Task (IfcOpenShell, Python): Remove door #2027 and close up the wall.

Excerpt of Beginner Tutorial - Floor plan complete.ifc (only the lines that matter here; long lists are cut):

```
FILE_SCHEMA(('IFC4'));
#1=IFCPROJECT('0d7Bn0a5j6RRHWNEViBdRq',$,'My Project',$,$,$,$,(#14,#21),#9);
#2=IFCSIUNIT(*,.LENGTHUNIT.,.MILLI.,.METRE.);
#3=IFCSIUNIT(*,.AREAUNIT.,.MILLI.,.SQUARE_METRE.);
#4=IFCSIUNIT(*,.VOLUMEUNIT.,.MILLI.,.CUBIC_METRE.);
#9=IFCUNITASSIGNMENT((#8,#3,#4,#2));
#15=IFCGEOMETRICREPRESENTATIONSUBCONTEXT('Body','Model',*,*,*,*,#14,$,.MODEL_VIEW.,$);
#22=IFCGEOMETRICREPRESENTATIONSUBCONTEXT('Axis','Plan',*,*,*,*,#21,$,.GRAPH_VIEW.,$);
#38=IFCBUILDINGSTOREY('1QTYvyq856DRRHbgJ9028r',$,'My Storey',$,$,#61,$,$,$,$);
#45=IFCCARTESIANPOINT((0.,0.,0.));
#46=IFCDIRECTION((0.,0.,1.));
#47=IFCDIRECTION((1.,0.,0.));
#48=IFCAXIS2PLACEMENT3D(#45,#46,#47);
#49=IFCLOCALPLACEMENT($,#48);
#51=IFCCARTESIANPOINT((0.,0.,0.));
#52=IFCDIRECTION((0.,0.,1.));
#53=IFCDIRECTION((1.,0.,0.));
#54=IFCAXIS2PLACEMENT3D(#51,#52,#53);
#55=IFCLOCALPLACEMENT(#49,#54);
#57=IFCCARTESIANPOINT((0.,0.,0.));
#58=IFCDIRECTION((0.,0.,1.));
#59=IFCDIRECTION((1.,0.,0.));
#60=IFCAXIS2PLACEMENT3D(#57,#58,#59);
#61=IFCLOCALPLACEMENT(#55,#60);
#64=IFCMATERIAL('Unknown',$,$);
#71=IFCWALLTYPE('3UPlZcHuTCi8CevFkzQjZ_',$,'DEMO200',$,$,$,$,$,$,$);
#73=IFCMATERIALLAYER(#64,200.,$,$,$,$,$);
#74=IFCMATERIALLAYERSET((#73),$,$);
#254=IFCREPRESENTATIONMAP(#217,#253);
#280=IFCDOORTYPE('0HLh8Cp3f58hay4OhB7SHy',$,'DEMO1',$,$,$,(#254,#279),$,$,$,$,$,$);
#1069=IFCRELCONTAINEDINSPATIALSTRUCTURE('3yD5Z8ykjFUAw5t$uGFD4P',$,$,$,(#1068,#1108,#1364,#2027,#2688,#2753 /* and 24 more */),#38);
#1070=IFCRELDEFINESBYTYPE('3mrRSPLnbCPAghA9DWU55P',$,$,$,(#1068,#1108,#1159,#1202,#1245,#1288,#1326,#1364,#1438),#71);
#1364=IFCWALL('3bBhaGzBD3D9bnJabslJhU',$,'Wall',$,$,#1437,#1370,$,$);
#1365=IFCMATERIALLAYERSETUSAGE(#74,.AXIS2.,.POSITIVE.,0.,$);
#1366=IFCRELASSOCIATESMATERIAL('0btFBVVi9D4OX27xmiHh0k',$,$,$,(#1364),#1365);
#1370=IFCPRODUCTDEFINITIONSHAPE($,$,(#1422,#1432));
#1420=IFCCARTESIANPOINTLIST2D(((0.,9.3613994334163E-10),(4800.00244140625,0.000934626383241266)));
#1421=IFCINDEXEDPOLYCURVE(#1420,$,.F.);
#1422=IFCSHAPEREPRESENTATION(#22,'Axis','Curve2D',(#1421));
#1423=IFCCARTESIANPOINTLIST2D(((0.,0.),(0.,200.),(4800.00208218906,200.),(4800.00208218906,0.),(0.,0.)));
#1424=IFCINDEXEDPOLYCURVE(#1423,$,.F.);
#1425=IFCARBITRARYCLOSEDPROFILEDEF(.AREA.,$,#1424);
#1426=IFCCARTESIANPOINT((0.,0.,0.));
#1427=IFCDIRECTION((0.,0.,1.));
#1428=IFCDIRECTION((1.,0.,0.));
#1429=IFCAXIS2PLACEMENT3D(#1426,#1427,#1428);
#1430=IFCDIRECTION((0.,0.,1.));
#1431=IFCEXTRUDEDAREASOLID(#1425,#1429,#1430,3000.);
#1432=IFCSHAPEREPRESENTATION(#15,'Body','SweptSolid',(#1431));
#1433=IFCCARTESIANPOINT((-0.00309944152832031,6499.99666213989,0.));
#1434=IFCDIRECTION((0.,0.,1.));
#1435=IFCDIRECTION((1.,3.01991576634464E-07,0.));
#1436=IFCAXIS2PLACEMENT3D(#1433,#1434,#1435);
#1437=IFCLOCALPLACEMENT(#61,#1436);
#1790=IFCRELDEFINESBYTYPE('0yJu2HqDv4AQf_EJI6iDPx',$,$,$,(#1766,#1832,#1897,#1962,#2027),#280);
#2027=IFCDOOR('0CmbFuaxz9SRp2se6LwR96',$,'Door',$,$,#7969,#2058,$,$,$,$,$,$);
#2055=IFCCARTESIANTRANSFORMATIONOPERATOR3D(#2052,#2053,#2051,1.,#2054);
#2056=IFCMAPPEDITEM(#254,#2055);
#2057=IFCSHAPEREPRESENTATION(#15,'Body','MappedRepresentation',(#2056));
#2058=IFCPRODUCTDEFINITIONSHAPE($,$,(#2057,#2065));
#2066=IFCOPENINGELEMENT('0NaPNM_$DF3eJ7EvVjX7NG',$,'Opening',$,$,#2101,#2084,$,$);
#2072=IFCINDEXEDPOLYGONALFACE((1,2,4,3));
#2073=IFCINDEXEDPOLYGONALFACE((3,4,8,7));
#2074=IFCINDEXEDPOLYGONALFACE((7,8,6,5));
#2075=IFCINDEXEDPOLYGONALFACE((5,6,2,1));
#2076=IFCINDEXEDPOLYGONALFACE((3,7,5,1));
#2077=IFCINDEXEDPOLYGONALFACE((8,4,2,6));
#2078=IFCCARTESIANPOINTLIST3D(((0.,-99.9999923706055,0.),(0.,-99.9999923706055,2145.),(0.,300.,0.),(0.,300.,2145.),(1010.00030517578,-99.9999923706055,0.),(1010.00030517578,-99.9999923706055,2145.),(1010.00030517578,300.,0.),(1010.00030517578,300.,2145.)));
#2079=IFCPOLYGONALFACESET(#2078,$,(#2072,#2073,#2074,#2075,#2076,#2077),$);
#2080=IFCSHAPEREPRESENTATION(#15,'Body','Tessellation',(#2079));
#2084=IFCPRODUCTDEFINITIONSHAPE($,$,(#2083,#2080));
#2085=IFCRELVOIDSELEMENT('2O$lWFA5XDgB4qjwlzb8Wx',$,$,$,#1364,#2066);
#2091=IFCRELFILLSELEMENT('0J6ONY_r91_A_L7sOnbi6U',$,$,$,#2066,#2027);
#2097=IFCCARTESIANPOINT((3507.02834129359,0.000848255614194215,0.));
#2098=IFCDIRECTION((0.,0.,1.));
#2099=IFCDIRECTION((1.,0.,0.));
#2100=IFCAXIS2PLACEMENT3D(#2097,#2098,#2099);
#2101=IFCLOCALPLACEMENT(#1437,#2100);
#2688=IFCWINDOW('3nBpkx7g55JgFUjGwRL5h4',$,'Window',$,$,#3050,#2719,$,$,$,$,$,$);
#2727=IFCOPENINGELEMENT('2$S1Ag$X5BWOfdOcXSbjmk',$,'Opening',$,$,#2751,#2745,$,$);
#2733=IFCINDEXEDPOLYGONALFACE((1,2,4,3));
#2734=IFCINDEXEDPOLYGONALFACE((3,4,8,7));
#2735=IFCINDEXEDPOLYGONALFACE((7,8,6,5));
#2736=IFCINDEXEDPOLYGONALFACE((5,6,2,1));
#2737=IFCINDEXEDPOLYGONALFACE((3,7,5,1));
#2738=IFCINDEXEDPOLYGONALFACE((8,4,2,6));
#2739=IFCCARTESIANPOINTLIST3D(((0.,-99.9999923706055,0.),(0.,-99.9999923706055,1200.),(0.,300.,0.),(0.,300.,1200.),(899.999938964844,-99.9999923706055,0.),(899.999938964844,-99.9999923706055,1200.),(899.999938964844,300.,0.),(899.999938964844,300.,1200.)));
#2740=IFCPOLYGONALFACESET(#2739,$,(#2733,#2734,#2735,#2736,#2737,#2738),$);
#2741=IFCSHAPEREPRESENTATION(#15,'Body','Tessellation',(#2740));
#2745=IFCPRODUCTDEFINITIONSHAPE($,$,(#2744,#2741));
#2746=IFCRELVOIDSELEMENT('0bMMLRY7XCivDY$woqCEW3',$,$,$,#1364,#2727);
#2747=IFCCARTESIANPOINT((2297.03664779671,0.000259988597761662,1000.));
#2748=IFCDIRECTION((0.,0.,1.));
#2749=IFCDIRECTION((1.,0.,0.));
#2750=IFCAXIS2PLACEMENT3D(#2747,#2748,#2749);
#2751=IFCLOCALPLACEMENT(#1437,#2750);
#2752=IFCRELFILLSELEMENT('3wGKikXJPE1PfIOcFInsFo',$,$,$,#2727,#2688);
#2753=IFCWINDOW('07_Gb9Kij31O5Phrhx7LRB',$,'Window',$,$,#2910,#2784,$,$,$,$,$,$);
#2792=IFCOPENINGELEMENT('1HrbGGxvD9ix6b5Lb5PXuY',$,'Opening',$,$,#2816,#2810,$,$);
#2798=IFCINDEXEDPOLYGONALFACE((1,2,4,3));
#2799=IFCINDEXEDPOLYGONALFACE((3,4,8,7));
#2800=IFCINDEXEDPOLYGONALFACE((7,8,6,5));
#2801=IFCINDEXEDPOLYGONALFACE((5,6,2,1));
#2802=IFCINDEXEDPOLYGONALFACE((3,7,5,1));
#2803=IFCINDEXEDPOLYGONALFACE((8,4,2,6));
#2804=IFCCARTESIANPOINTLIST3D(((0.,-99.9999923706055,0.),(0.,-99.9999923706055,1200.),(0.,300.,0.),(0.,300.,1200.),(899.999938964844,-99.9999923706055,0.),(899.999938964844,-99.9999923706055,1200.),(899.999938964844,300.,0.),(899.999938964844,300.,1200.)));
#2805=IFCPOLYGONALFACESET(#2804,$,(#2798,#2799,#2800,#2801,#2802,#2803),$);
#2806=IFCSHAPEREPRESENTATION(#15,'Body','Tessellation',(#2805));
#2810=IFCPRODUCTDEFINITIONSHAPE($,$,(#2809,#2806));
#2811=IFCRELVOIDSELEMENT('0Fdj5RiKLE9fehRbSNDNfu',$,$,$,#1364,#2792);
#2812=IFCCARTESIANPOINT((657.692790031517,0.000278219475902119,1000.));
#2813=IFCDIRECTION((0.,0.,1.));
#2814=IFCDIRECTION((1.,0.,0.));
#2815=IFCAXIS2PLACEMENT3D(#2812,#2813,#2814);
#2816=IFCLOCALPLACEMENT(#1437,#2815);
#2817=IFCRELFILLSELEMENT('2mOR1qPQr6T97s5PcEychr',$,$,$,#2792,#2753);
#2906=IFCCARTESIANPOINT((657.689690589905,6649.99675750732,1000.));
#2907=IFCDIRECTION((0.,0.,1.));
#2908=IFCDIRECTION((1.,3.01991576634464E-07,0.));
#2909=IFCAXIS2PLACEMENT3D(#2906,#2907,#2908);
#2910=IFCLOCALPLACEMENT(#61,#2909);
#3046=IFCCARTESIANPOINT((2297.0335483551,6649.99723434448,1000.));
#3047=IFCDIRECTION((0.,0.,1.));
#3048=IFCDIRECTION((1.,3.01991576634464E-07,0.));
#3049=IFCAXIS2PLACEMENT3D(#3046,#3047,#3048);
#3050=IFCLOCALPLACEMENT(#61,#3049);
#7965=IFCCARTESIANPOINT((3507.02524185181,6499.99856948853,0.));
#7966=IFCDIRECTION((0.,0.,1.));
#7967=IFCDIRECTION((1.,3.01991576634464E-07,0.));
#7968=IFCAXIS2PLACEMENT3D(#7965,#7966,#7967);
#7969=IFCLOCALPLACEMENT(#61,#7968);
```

```python
import ifcopenshell
import ifcopenshell.api.feature
import ifcopenshell.api.root
import ifcopenshell.geom
import ifcopenshell.util.shape

model = ifcopenshell.open("Beginner Tutorial - Floor plan complete.ifc")
settings = ifcopenshell.geom.settings()


def volume(element):
    """Net volume in cubic metres, openings subtracted."""
    shape = ifcopenshell.geom.create_shape(settings, element)
    return ifcopenshell.util.shape.get_volume(shape.geometry)


door = model.by_guid("0CmbFuaxz9SRp2se6LwR96")
opening = door.FillsVoids[0].RelatingOpeningElement
wall = opening.VoidsElements[0].RelatingBuildingElement
before = volume(wall)

ifcopenshell.api.root.remove_product(model, product=door)
ifcopenshell.api.feature.remove_feature(model, feature=opening)

after = volume(wall)

print(f"wall volume {before:.3f} -> {after:.3f} m3")

model.write("Beginner Tutorial - Floor plan complete_updated.ifc")
```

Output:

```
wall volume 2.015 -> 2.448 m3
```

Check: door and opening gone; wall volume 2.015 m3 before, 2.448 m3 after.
